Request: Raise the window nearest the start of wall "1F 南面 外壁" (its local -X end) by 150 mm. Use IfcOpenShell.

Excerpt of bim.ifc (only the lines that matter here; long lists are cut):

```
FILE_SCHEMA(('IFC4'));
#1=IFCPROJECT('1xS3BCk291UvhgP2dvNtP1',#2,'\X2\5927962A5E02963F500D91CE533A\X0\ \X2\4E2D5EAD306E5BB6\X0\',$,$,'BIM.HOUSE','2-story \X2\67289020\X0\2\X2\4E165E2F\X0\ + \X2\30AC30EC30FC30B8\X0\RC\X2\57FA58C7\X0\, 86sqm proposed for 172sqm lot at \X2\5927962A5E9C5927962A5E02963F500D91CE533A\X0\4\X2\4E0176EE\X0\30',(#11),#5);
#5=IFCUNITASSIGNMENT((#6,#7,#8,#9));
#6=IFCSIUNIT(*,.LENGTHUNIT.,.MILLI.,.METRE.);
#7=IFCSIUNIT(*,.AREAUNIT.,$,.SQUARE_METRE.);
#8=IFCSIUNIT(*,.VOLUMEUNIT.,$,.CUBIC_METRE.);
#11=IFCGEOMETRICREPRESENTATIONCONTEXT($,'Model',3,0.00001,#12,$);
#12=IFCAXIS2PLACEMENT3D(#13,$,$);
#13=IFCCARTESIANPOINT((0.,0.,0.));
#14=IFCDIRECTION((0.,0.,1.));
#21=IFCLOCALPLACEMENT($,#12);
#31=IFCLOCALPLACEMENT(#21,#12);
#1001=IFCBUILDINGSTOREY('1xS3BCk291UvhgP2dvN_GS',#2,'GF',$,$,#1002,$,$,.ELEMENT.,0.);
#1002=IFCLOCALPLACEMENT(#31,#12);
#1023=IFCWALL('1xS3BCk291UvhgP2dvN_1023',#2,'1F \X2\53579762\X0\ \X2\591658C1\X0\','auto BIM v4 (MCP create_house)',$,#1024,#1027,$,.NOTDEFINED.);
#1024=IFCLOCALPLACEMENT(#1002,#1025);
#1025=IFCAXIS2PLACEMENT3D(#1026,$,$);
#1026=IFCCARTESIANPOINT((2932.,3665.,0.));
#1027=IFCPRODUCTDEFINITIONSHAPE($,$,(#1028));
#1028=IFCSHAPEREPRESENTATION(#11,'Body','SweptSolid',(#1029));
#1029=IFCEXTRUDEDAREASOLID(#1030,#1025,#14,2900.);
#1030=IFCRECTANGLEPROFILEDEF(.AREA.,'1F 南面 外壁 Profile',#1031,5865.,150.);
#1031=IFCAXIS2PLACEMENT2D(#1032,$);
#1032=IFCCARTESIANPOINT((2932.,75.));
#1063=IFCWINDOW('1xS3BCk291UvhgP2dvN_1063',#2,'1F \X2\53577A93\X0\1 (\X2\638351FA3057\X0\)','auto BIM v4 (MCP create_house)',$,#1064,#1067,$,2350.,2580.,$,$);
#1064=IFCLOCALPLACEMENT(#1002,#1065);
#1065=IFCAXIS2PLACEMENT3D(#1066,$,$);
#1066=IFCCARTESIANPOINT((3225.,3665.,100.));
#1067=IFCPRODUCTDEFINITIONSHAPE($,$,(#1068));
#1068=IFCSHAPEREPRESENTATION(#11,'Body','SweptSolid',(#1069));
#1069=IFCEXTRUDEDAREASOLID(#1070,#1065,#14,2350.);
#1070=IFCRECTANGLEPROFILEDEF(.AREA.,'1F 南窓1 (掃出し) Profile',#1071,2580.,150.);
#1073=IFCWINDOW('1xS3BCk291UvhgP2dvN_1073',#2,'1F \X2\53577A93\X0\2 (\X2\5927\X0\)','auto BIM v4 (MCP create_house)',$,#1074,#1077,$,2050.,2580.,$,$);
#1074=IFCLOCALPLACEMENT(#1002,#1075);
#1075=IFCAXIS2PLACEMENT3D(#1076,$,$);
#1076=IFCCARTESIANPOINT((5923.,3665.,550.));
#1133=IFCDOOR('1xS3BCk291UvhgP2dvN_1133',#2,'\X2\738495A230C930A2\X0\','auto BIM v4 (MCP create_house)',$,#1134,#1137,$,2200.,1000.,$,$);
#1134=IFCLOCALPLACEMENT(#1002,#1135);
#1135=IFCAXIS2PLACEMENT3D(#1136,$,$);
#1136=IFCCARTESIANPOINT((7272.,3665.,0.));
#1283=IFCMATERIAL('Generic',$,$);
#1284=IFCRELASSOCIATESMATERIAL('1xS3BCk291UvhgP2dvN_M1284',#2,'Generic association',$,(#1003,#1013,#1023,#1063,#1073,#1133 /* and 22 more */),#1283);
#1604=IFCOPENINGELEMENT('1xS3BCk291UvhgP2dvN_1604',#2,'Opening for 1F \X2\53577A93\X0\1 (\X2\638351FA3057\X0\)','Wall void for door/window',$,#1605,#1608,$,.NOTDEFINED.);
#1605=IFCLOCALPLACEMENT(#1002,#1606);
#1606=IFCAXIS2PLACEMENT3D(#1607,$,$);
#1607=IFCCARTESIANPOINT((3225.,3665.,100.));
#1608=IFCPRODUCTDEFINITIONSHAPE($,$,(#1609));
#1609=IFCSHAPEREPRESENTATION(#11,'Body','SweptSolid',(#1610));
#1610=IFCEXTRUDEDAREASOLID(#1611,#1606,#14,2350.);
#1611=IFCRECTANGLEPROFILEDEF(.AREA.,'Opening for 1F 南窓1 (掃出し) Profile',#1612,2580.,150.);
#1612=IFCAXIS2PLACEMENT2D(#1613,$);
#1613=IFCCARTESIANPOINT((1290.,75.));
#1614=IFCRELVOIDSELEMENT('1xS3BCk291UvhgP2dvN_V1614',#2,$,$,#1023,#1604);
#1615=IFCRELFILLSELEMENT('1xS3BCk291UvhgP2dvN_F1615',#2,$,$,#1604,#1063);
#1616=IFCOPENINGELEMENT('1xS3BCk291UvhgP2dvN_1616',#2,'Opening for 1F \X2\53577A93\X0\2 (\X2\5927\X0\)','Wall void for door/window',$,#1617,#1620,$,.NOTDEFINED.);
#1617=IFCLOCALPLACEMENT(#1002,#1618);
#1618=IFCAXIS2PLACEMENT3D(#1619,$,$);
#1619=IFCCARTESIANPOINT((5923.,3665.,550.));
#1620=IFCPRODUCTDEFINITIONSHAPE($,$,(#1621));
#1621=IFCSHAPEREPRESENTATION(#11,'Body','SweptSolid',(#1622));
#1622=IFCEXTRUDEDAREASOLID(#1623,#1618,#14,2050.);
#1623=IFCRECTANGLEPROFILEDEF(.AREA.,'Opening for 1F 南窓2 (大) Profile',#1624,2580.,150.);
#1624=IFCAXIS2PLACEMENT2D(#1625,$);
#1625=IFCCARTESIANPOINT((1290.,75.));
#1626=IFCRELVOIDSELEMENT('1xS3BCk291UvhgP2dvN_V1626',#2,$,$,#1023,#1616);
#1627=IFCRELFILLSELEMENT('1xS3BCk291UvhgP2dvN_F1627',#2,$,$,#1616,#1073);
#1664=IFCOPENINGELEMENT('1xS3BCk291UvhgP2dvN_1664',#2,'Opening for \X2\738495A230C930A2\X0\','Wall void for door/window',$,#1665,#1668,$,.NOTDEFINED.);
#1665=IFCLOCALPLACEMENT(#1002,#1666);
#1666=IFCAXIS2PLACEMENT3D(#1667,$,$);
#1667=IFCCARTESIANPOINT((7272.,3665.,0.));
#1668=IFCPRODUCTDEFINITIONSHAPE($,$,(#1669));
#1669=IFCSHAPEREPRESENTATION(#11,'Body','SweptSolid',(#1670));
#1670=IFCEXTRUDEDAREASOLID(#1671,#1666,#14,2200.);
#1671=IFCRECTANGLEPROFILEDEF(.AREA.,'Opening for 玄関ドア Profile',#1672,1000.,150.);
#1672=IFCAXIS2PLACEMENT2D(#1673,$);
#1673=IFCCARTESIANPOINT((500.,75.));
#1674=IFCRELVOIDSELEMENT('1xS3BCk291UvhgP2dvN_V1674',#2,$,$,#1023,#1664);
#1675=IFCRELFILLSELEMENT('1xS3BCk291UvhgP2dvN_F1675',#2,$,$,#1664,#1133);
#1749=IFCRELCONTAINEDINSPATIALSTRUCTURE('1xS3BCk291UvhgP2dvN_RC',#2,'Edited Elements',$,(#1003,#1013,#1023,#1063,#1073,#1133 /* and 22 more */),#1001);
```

```python
import numpy as np
import ifcopenshell
import ifcopenshell.api.geometry
import ifcopenshell.util.placement
import ifcopenshell.util.unit

model = ifcopenshell.open("bim.ifc")
unit_scale = ifcopenshell.util.unit.calculate_unit_scale(model)

window = model.by_guid("1xS3BCk291UvhgP2dvN_1063")
opening = window.FillsVoids[0].RelatingOpeningElement
dz = 0.15 / unit_scale

shift = np.array([0.0, 0.0, dz])
# The window is not placed relative to its opening, so move both.
for product in (opening, window):
    matrix = ifcopenshell.util.placement.get_local_placement(product.ObjectPlacement)
    matrix[:3, 3] += shift
    ifcopenshell.api.geometry.edit_object_placement(model, product=product, matrix=matrix, is_si=False)

print(f"moved by {dz * unit_scale:+.3f} m")

model.write("bim_updated.ifc")
```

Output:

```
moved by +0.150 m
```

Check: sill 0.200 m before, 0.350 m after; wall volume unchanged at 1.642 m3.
